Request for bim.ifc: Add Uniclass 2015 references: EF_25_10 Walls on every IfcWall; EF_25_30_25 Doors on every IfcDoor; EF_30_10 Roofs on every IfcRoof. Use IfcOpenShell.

First a look at what the model holds.

```python
import ifcopenshell

model = ifcopenshell.open("bim.ifc")
print(model.schema)
print("classifications:", [c.Name for c in model.by_type("IfcClassification")])
for ifc_class in ("IfcDoor", "IfcRoof", "IfcStair", "IfcWall", "IfcWindow"):
    print(ifc_class, len(model.by_type(ifc_class)))
```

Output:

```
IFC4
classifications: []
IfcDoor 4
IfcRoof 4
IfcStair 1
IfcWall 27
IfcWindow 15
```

```python
import ifcopenshell
import ifcopenshell.api.classification

model = ifcopenshell.open("bim.ifc")

system = ifcopenshell.api.classification.add_classification(model, classification="Uniclass 2015")

codes = {
    "IfcWall": ("EF_25_10", "Walls"),
    "IfcDoor": ("EF_25_30_25", "Doors"),
    "IfcRoof": ("EF_30_10", "Roofs"),
}
for ifc_class, (code, name) in codes.items():
    products = model.by_type(ifc_class)
    ifcopenshell.api.classification.add_reference(
        model, products=products, classification=system, identification=code, name=name
    )
    print(code, len(products))

model.write("bim_edited.ifc")
```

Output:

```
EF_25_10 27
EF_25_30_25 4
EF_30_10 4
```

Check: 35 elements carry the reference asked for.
